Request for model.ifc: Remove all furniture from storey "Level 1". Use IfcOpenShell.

First a look at what the model holds.

```python
import ifcopenshell
import ifcopenshell.util.element

model = ifcopenshell.open("model.ifc")
print(model.schema)
storey = next(s for s in model.by_type("IfcBuildingStorey") if s.Name == "Level 1")
furniture = [e for e in ifcopenshell.util.element.get_decomposition(storey) if e.is_a("IfcFurnishingElement")]
seen = {}
for e in furniture:
    element_type = ifcopenshell.util.element.get_type(e)
    name = element_type.Name if element_type not in (None, e) else None
    seen[name] = seen.get(name, 0) + 1
for name, count in sorted(seen.items(), key=str):
    print(count, "x", name)
```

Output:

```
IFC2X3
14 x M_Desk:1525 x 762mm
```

```python
import ifcopenshell
import ifcopenshell.api.root
import ifcopenshell.util.element

model = ifcopenshell.open("model.ifc")

storey = next(s for s in model.by_type("IfcBuildingStorey") if s.Name == "Level 1")
furniture = [e for e in ifcopenshell.util.element.get_decomposition(storey) if e.is_a("IfcFurnishingElement")]

for e in furniture:
    ifcopenshell.api.root.remove_product(model, product=e)
print(len(furniture), "removed")

model.write("model_rev.ifc")
```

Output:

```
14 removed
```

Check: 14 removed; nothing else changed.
